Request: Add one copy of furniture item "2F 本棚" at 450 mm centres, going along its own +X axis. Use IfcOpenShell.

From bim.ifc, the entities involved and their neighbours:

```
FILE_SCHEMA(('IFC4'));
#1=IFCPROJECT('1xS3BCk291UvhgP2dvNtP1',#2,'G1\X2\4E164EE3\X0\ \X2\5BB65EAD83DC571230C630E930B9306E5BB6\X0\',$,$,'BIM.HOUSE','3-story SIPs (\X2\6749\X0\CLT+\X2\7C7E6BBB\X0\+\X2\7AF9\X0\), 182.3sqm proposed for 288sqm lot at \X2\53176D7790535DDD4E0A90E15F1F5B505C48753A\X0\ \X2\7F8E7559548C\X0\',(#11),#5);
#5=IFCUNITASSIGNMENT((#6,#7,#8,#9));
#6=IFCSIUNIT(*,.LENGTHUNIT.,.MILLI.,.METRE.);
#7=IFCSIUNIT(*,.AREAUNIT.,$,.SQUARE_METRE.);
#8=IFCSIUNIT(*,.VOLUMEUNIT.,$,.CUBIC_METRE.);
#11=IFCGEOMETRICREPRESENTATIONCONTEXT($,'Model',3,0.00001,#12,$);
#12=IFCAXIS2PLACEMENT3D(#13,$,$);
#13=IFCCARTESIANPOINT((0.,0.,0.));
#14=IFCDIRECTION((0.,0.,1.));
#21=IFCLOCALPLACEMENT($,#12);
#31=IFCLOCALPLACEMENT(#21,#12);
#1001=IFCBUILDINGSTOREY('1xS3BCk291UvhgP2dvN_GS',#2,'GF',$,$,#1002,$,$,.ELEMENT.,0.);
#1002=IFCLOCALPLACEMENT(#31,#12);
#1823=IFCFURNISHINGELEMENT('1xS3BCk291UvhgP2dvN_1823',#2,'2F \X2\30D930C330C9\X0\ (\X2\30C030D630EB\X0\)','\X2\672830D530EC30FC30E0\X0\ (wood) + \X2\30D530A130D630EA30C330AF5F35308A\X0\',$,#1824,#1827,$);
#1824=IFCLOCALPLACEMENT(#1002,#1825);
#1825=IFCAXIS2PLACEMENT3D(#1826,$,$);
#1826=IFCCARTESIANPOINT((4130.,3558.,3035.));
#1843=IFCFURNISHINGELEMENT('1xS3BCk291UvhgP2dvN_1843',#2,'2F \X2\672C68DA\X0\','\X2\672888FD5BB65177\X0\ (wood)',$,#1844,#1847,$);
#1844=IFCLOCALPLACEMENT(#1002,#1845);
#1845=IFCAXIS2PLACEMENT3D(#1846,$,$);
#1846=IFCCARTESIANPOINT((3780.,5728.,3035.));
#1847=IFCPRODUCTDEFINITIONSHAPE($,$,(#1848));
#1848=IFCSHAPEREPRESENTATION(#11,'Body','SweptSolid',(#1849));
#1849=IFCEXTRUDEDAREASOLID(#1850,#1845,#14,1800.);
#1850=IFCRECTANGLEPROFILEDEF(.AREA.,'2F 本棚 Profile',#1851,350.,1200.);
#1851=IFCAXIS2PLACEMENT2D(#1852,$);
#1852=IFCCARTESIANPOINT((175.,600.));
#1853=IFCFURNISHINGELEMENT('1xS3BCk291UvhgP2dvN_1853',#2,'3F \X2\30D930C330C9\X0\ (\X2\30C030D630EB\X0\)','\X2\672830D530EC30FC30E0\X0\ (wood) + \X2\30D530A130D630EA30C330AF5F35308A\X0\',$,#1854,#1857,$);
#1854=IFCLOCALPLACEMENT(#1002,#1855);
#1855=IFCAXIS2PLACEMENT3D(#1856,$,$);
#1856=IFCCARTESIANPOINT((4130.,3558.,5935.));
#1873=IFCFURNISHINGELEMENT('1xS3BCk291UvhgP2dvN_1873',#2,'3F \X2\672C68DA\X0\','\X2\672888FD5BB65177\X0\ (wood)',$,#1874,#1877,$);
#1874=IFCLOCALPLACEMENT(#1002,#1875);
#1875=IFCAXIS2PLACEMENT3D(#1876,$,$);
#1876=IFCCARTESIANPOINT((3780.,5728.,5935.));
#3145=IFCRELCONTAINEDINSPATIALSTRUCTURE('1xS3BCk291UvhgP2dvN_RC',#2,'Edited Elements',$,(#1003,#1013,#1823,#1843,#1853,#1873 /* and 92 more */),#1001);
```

```python
import ifcopenshell
import ifcopenshell.api.geometry
import ifcopenshell.api.root
import ifcopenshell.util.element
import ifcopenshell.util.placement
import ifcopenshell.util.unit

model = ifcopenshell.open("bim.ifc")
unit_scale = ifcopenshell.util.unit.calculate_unit_scale(model)


def reuse_history(source, copy):
    """copy_class also copies each property set's owner history, people and application; keep the originals."""
    for rel in copy.IsDefinedBy:
        if rel.is_a("IfcRelDefinesByProperties") and (history := rel.RelatingPropertyDefinition.OwnerHistory):
            rel.RelatingPropertyDefinition.OwnerHistory = source.OwnerHistory
            ifcopenshell.util.element.remove_deep2(model, history)


source = model.by_guid("1xS3BCk291UvhgP2dvN_1843")
base = ifcopenshell.util.placement.get_local_placement(source.ObjectPlacement)
step = base[:3, 0] * 0.45 / unit_scale

for i in range(1, 2):
    copy = ifcopenshell.api.root.copy_class(model, product=source)
    copy.Representation = ifcopenshell.util.element.copy_deep(
        model, source.Representation, exclude=["IfcGeometricRepresentationContext", "IfcRepresentationMap"]
    )
    reuse_history(source, copy)
    matrix = base.copy()
    matrix[:3, 3] += i * step
    print("added at", matrix[:3, 3].round(3) + 0.0)
    ifcopenshell.api.geometry.edit_object_placement(model, product=copy, matrix=matrix, is_si=False)

model.write("bim_rev.ifc")
```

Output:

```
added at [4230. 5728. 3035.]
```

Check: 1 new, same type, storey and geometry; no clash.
